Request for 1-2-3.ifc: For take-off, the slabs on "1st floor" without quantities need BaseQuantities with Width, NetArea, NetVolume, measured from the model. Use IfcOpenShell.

First a look at what the model holds.

```python
import ifcopenshell
import ifcopenshell.util.element
import ifcopenshell.util.unit

model = ifcopenshell.open("1-2-3.ifc")
print(model.schema)
for unit_type in ("LENGTHUNIT", "AREAUNIT", "VOLUMEUNIT"):
    print(unit_type, ifcopenshell.util.unit.calculate_unit_scale(model, unit_type))
storey = next(s for s in model.by_type("IfcBuildingStorey") if s.Name == "1st floor")
slabs = [e for e in ifcopenshell.util.element.get_decomposition(storey) if e.is_a("IfcSlab")]
for e in sorted(slabs, key=lambda e: e.id()):
    print(e.id(), e.is_a(), e.Name, list(ifcopenshell.util.element.get_psets(e, qtos_only=True)), sep=" | ")
```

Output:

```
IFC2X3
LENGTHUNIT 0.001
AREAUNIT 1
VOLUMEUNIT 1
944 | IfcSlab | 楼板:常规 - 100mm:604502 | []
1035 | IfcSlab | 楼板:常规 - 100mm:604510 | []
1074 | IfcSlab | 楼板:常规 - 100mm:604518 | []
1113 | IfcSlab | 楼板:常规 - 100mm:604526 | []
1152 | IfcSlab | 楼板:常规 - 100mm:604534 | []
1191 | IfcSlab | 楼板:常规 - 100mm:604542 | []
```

```python
import ifcopenshell
import ifcopenshell.api.pset
import ifcopenshell.geom
import ifcopenshell.util.element
import ifcopenshell.util.shape
import ifcopenshell.util.unit

model = ifcopenshell.open("1-2-3.ifc")
unit_scale = ifcopenshell.util.unit.calculate_unit_scale(model)
area_scale = ifcopenshell.util.unit.calculate_unit_scale(model, "AREAUNIT")
volume_scale = ifcopenshell.util.unit.calculate_unit_scale(model, "VOLUMEUNIT")
settings = ifcopenshell.geom.settings()

storey = next(s for s in model.by_type("IfcBuildingStorey") if s.Name == "1st floor")
slabs = [e for e in ifcopenshell.util.element.get_decomposition(storey) if e.is_a("IfcSlab")]

for e in sorted(slabs, key=lambda e: e.id()):
    if ifcopenshell.util.element.get_psets(e, qtos_only=True, should_inherit=False):
        continue
    # Geometry comes back in metres, in the element's own axes.
    shape = ifcopenshell.geom.create_shape(settings, e)
    values = {
        "Width": ifcopenshell.util.shape.get_z(shape.geometry) / unit_scale,
        "NetArea": ifcopenshell.util.shape.get_footprint_area(shape.geometry) / area_scale,
        "NetVolume": ifcopenshell.util.shape.get_volume(shape.geometry) / volume_scale,
    }
    qto = ifcopenshell.api.pset.add_qto(model, product=e, name="BaseQuantities")
    ifcopenshell.api.pset.edit_qto(model, qto=qto, properties=values)
    print(e.id(), {k: round(v, 3) for k, v in values.items()})

model.write("1-2-3_updated.ifc")
```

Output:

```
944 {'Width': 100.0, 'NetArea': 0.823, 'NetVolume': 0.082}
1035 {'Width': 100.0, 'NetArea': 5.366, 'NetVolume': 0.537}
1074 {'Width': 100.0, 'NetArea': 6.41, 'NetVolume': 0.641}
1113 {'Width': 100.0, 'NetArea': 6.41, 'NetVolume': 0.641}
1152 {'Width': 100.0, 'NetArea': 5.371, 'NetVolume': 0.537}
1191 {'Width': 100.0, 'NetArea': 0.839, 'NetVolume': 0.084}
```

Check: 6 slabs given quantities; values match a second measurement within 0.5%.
